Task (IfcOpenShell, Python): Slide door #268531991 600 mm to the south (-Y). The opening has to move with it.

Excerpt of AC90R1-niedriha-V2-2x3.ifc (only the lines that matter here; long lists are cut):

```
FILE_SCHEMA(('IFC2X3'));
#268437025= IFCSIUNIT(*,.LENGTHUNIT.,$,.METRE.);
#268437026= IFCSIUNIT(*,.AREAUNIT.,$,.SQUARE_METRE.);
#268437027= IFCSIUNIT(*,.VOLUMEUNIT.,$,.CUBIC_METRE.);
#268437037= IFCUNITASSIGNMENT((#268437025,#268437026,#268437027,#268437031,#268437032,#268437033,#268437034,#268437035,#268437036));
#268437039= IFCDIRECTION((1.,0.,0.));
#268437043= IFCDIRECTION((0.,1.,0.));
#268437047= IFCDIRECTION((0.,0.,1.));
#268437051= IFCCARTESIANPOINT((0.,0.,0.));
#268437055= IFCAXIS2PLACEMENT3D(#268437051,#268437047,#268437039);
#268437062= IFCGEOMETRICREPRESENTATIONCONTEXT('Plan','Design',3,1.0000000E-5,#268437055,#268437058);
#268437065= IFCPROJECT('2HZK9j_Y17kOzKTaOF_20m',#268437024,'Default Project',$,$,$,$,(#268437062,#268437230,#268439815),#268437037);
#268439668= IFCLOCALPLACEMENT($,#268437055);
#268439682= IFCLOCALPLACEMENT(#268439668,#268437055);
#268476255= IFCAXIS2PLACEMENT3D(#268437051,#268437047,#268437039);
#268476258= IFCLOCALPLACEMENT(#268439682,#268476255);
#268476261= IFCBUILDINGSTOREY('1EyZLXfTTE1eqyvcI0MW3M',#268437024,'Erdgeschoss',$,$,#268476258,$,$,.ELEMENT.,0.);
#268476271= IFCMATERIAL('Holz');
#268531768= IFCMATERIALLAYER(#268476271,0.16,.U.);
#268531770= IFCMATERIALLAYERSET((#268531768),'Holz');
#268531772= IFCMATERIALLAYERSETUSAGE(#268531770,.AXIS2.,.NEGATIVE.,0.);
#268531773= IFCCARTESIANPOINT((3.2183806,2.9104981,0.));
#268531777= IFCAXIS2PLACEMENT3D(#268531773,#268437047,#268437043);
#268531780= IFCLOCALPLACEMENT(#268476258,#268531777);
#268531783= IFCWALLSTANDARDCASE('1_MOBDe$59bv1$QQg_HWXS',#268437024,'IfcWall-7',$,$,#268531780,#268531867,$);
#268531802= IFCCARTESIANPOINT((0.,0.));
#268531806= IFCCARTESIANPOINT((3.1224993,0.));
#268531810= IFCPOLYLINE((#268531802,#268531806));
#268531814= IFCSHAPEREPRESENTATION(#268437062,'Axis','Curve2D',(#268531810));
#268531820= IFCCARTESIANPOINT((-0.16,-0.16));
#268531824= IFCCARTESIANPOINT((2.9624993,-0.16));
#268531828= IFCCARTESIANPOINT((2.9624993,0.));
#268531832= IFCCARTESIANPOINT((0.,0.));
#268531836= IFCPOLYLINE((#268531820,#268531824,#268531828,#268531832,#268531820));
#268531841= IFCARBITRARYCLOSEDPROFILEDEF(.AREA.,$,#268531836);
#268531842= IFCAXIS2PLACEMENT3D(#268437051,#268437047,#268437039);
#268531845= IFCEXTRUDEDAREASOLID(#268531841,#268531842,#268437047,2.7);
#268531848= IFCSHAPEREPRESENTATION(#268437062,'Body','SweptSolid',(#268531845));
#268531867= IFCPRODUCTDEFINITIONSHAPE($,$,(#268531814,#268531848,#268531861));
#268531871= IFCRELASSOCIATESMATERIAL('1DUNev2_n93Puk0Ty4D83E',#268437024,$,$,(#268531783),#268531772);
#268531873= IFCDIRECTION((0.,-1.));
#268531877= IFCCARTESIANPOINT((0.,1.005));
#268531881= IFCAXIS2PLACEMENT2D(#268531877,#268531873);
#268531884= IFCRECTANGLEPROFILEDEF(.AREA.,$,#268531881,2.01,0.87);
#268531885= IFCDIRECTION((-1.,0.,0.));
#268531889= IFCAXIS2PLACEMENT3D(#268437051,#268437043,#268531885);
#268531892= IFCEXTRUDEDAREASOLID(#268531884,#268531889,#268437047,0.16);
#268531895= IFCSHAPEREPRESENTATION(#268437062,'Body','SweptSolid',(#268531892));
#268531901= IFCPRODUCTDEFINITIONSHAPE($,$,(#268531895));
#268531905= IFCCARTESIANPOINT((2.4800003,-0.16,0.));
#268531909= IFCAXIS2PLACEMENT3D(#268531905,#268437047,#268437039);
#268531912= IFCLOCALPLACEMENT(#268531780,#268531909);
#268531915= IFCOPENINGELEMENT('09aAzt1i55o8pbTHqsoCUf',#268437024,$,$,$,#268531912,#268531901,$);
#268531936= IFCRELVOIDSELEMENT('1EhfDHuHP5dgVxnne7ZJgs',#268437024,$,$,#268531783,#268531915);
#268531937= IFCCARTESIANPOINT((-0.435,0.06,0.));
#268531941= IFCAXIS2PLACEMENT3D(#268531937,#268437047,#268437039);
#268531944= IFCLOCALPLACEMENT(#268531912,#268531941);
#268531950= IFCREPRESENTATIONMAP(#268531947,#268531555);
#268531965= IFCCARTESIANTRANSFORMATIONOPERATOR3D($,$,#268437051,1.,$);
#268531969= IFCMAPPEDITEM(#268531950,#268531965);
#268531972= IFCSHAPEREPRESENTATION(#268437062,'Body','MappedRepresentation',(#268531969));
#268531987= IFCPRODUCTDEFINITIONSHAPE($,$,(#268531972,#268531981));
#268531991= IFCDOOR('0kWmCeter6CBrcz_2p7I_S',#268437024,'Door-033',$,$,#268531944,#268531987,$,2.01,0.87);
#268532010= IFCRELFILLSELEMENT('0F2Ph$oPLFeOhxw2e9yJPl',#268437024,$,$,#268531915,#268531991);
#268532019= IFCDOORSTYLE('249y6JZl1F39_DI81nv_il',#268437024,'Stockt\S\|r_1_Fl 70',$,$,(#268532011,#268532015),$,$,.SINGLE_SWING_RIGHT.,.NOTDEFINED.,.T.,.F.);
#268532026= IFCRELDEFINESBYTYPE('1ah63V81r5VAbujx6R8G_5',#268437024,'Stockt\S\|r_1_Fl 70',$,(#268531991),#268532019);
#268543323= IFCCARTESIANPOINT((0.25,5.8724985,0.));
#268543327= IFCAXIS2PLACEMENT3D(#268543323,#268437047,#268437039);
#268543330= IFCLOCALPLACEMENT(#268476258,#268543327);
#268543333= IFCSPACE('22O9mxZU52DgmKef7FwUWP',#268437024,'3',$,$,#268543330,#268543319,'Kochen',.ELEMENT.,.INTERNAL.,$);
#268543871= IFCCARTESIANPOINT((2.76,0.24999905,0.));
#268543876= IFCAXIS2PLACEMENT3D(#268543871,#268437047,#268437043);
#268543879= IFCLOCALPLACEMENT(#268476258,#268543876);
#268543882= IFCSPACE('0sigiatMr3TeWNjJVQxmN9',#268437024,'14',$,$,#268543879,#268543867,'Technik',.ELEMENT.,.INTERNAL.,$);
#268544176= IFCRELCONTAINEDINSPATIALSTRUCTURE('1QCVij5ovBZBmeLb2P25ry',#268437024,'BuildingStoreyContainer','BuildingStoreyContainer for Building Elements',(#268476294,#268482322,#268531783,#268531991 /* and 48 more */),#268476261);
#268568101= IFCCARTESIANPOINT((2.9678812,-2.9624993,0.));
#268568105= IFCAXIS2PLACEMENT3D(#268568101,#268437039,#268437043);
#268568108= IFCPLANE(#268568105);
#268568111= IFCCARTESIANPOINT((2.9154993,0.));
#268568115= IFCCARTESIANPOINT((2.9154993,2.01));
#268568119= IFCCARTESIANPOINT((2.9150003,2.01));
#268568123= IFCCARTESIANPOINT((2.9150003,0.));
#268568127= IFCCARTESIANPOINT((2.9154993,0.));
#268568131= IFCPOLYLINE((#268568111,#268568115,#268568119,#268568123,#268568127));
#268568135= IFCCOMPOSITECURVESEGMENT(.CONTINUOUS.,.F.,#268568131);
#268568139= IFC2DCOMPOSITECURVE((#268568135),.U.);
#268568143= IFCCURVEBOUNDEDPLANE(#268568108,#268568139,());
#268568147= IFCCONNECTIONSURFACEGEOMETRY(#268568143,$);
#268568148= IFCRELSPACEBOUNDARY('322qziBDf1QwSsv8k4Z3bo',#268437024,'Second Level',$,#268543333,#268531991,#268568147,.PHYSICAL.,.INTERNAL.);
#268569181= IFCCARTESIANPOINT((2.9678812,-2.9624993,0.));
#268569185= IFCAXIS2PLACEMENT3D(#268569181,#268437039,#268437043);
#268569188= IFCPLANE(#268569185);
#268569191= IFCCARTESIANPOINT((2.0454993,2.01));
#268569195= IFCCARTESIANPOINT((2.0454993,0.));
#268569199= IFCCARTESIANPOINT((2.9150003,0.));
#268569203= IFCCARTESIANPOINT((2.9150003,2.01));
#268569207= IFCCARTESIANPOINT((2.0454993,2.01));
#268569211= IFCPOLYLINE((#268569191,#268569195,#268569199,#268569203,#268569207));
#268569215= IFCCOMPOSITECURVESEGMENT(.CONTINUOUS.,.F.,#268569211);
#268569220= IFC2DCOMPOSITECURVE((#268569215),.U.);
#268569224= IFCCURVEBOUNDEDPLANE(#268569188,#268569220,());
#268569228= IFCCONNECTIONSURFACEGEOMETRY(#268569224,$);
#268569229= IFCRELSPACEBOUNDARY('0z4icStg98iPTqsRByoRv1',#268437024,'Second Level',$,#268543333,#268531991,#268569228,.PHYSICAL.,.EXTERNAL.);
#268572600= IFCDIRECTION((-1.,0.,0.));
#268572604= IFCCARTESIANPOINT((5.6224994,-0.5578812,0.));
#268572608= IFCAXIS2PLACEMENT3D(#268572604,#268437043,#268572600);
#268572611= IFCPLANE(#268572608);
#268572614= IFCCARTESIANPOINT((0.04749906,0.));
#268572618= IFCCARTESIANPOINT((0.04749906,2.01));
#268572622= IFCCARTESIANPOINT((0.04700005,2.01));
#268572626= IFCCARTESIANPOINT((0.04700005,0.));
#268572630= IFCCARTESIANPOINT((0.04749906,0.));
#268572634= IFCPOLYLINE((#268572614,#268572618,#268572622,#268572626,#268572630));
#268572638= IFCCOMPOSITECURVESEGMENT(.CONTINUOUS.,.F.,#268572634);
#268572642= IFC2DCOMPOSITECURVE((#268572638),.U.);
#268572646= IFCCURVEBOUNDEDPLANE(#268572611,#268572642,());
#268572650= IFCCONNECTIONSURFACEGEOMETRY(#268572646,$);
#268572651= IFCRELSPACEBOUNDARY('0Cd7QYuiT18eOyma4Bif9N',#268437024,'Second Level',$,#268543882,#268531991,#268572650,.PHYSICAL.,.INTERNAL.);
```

```python
import numpy as np
import ifcopenshell
import ifcopenshell.api.geometry
import ifcopenshell.util.placement
import ifcopenshell.util.unit

model = ifcopenshell.open("AC90R1-niedriha-V2-2x3.ifc")
unit_scale = ifcopenshell.util.unit.calculate_unit_scale(model)

door = model.by_guid("0kWmCeter6CBrcz_2p7I_S")
opening = door.FillsVoids[0].RelatingOpeningElement
wall = opening.VoidsElements[0].RelatingBuildingElement

wall_matrix = ifcopenshell.util.placement.get_local_placement(wall.ObjectPlacement)
shift = wall_matrix[:3, 0] * -0.6 / unit_scale
before = ifcopenshell.util.placement.get_local_placement(door.ObjectPlacement)[:3, 3].copy()

# The door is placed relative to its opening, so it follows when the opening moves.
matrix = ifcopenshell.util.placement.get_local_placement(opening.ObjectPlacement)
matrix[:3, 3] += shift
ifcopenshell.api.geometry.edit_object_placement(
    model, product=opening, matrix=matrix, is_si=False, should_transform_children=True
)

# Space boundary surfaces are stored in each space's coordinates; move them too.
for rel in door.ProvidesBoundaries:
    if not rel.ConnectionGeometry:
        continue
    surface = rel.ConnectionGeometry.SurfaceOnRelatingElement.BasisSurface
    space_matrix = ifcopenshell.util.placement.get_local_placement(rel.RelatingSpace.ObjectPlacement)
    point = np.array(surface.Position.Location.Coordinates) + space_matrix[:3, :3].T @ shift
    surface.Position = model.createIfcAxis2Placement3D(
        model.createIfcCartesianPoint(point.tolist()), surface.Position.Axis, surface.Position.RefDirection
    )

after = ifcopenshell.util.placement.get_local_placement(door.ObjectPlacement)[:3, 3]
print("door moved by", (after - before).round(3) + 0.0)

model.write("AC90R1-niedriha-V2-2x3_rev.ifc")
```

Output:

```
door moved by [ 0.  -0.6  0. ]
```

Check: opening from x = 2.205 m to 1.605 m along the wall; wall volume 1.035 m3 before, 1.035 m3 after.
